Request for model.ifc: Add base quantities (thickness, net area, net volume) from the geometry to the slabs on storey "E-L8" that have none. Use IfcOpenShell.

First a look at what the model holds.

```python
import ifcopenshell
import ifcopenshell.util.element
import ifcopenshell.util.unit

model = ifcopenshell.open("model.ifc")
print(model.schema)
for unit_type in ("LENGTHUNIT", "AREAUNIT", "VOLUMEUNIT"):
    print(unit_type, ifcopenshell.util.unit.calculate_unit_scale(model, unit_type))
storey = next(s for s in model.by_type("IfcBuildingStorey") if s.Name == "E-L8")
slabs = [e for e in ifcopenshell.util.element.get_decomposition(storey) if e.is_a("IfcSlab")]
for e in sorted(slabs, key=lambda e: e.id()):
    print(e.id(), e.is_a(), e.Name, list(ifcopenshell.util.element.get_psets(e, qtos_only=True)), sep=" | ")
```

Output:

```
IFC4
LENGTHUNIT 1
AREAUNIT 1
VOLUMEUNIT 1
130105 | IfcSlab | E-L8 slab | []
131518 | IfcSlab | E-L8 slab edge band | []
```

```python
import ifcopenshell
import ifcopenshell.api.pset
import ifcopenshell.geom
import ifcopenshell.util.element
import ifcopenshell.util.shape
import ifcopenshell.util.unit

model = ifcopenshell.open("model.ifc")
unit_scale = ifcopenshell.util.unit.calculate_unit_scale(model)
area_scale = ifcopenshell.util.unit.calculate_unit_scale(model, "AREAUNIT")
volume_scale = ifcopenshell.util.unit.calculate_unit_scale(model, "VOLUMEUNIT")
settings = ifcopenshell.geom.settings()

storey = next(s for s in model.by_type("IfcBuildingStorey") if s.Name == "E-L8")
slabs = [e for e in ifcopenshell.util.element.get_decomposition(storey) if e.is_a("IfcSlab")]

for e in sorted(slabs, key=lambda e: e.id()):
    if ifcopenshell.util.element.get_psets(e, qtos_only=True, should_inherit=False):
        continue
    # Geometry comes back in metres, in the element's own axes.
    shape = ifcopenshell.geom.create_shape(settings, e)
    values = {
        "Width": ifcopenshell.util.shape.get_z(shape.geometry) / unit_scale,
        "NetArea": ifcopenshell.util.shape.get_footprint_area(shape.geometry) / area_scale,
        "NetVolume": ifcopenshell.util.shape.get_volume(shape.geometry) / volume_scale,
    }
    qto = ifcopenshell.api.pset.add_qto(model, product=e, name="Qto_SlabBaseQuantities")
    ifcopenshell.api.pset.edit_qto(model, qto=qto, properties=values)
    print(e.id(), {k: round(v, 3) for k, v in values.items()})

model.write("model_updated.ifc")
```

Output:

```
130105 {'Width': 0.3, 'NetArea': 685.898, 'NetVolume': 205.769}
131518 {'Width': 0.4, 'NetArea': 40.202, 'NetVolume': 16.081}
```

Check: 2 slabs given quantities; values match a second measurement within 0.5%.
